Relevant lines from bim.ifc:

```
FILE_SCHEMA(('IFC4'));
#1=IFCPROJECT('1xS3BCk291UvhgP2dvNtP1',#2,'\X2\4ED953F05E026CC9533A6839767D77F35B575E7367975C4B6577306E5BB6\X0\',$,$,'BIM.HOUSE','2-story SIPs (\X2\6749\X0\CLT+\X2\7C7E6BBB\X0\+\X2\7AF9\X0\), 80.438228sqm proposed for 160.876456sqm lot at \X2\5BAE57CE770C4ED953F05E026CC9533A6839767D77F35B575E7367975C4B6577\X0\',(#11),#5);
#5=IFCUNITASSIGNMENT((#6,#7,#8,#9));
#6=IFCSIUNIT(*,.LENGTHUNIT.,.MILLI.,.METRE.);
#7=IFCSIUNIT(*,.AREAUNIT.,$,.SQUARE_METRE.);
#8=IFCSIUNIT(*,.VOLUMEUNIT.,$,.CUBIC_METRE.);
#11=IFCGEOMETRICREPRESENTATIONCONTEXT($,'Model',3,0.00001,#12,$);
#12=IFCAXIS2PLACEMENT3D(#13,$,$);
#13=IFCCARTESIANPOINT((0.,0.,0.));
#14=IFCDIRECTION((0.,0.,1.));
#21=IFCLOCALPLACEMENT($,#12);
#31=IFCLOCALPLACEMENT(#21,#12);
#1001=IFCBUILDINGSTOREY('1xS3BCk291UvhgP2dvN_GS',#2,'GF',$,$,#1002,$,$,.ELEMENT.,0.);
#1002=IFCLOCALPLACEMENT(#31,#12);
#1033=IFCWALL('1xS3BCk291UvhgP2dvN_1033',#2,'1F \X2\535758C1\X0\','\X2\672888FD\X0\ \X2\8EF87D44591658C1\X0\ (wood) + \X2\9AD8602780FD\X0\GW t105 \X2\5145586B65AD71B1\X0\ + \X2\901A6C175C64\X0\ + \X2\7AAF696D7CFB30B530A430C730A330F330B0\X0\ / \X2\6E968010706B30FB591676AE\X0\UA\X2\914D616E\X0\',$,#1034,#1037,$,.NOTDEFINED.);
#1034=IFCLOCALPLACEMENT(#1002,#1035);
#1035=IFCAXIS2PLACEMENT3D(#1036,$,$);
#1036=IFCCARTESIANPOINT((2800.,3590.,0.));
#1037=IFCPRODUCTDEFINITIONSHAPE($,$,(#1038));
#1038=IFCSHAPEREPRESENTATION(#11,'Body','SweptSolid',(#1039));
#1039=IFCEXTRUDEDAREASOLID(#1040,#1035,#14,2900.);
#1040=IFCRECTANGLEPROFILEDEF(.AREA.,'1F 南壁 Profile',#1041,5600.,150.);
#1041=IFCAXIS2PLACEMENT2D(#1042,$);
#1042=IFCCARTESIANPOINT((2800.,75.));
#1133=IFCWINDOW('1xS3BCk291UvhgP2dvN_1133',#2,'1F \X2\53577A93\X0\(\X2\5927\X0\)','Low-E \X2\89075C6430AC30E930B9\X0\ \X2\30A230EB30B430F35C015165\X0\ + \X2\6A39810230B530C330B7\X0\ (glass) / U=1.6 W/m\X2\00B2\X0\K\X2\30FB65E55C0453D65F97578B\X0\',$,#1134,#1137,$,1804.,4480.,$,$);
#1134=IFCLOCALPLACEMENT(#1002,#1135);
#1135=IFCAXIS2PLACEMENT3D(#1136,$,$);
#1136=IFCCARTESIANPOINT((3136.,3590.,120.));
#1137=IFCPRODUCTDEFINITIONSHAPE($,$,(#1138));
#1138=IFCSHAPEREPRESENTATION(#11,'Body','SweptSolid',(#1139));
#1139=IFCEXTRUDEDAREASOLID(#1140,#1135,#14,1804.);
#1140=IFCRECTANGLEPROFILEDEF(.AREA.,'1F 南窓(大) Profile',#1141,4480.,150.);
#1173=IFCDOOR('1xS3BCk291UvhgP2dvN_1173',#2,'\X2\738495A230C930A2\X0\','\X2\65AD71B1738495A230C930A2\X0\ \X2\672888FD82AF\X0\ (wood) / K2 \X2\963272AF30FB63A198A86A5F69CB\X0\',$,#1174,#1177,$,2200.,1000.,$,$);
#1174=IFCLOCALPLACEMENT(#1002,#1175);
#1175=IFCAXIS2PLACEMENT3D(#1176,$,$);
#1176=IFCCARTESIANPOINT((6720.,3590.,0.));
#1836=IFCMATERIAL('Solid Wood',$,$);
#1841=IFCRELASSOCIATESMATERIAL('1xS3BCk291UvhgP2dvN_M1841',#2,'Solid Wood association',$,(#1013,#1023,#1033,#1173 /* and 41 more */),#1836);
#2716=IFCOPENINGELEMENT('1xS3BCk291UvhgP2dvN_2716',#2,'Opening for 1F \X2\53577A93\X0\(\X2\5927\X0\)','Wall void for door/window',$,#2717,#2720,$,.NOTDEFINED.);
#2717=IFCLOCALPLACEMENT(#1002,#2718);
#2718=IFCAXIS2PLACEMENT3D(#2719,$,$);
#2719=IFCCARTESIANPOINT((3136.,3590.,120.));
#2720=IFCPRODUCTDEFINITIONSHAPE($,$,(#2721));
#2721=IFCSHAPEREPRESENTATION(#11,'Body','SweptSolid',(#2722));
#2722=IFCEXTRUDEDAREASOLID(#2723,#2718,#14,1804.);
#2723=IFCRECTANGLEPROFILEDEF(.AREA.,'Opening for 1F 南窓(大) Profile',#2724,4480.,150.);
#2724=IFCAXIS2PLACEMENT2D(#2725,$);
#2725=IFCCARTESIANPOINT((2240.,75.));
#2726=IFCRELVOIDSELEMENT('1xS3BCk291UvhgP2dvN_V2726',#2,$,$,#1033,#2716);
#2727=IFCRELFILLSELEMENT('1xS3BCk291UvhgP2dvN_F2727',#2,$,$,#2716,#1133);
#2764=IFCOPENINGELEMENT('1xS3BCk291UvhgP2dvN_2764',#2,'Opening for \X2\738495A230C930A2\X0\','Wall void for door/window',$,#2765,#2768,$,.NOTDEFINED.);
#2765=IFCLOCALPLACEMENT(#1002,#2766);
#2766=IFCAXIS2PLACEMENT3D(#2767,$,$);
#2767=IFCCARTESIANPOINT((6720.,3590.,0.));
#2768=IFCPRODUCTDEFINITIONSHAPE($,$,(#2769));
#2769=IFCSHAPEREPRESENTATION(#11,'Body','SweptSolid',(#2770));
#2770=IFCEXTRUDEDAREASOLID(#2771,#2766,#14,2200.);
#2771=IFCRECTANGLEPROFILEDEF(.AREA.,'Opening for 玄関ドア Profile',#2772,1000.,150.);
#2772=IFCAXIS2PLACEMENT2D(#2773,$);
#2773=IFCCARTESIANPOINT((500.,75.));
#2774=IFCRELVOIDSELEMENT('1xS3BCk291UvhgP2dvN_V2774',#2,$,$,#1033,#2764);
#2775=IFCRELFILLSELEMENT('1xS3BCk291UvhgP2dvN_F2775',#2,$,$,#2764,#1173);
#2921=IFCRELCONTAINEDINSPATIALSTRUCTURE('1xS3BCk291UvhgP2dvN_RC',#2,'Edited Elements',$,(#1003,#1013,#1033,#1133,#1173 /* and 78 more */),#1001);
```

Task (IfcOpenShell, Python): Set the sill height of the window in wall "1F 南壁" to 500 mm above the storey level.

```python
import numpy as np
import ifcopenshell
import ifcopenshell.api.geometry
import ifcopenshell.geom
import ifcopenshell.util.element
import ifcopenshell.util.placement
import ifcopenshell.util.shape
import ifcopenshell.util.unit

model = ifcopenshell.open("bim.ifc")
unit_scale = ifcopenshell.util.unit.calculate_unit_scale(model)

window = model.by_guid("1xS3BCk291UvhgP2dvN_1133")
opening = window.FillsVoids[0].RelatingOpeningElement
storey = ifcopenshell.util.element.get_container(window, ifc_class="IfcBuildingStorey")
level = ifcopenshell.util.placement.get_local_placement(storey.ObjectPlacement)[2, 3]

# The opening's origin need not be at the sill, so measure its lowest point.
shape = ifcopenshell.geom.create_shape(ifcopenshell.geom.settings(), opening)
bottom = ifcopenshell.util.shape.get_shape_bottom_elevation(shape, shape.geometry) / unit_scale
dz = level + 0.5 / unit_scale - bottom

shift = np.array([0.0, 0.0, dz])
# The window is not placed relative to its opening, so move both.
for product in (opening, window):
    matrix = ifcopenshell.util.placement.get_local_placement(product.ObjectPlacement)
    matrix[:3, 3] += shift
    ifcopenshell.api.geometry.edit_object_placement(model, product=product, matrix=matrix, is_si=False)

print(f"moved by {dz * unit_scale:+.3f} m")

model.write("bim_v2.ifc")
```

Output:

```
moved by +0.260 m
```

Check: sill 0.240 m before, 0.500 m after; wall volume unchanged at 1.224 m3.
